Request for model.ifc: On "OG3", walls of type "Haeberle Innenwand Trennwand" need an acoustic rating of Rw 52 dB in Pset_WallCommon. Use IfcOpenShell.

First a look at what the model holds.

```python
import ifcopenshell
import ifcopenshell.util.element

model = ifcopenshell.open("model.ifc")
print(model.schema)
storey = next(s for s in model.by_type("IfcBuildingStorey") if s.Name == "OG3")
walls = [e for e in ifcopenshell.util.element.get_decomposition(storey) if e.is_a("IfcWall")]
seen = {}
for e in walls:
    element_type = ifcopenshell.util.element.get_type(e)
    key = (element_type.Name if element_type != e and element_type else None, ifcopenshell.util.element.get_pset(e, "Pset_WallCommon", "AcousticRating"))
    seen[key] = seen.get(key, 0) + 1
for (name, value), count in sorted(seen.items(), key=str):
    print(count, "x", name, "|", value)
```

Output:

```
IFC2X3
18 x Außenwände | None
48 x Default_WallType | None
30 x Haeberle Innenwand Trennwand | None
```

```python
import ifcopenshell
import ifcopenshell.api.pset
import ifcopenshell.util.element

model = ifcopenshell.open("model.ifc")

storey = next(s for s in model.by_type("IfcBuildingStorey") if s.Name == "OG3")
walls = [e for e in ifcopenshell.util.element.get_decomposition(storey) if e.is_a("IfcWall")]

count = 0
for e in walls:
    element_type = ifcopenshell.util.element.get_type(e)
    if element_type in (None, e) or element_type.Name != "Haeberle Innenwand Trennwand":
        continue
    # add_pset returns the element's existing set when there is one.
    pset = ifcopenshell.api.pset.add_pset(model, product=e, name="Pset_WallCommon")
    ifcopenshell.api.pset.edit_pset(model, pset=pset, properties={"AcousticRating": "Rw 52 dB"})
    count += 1

print(count, "walls updated")

model.write("model_v2.ifc")
```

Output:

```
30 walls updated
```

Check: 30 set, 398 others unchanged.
